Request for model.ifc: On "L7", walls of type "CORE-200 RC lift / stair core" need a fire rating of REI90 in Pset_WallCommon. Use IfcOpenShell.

First a look at what the model holds.

```python
import ifcopenshell
import ifcopenshell.util.element

model = ifcopenshell.open("model.ifc")
print(model.schema)
storey = next(s for s in model.by_type("IfcBuildingStorey") if s.Name == "L7")
walls = [e for e in ifcopenshell.util.element.get_decomposition(storey) if e.is_a("IfcWall")]
seen = {}
for e in walls:
    element_type = ifcopenshell.util.element.get_type(e)
    key = (element_type.Name if element_type != e and element_type else None, ifcopenshell.util.element.get_pset(e, "Pset_WallCommon", "FireRating"))
    seen[key] = seen.get(key, 0) + 1
for (name, value), count in sorted(seen.items(), key=str):
    print(count, "x", name, "|", value)
```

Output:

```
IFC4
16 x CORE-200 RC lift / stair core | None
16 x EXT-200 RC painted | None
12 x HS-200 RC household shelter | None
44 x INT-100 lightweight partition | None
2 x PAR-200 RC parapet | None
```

```python
import ifcopenshell
import ifcopenshell.api.pset
import ifcopenshell.util.element

model = ifcopenshell.open("model.ifc")

storey = next(s for s in model.by_type("IfcBuildingStorey") if s.Name == "L7")
walls = [e for e in ifcopenshell.util.element.get_decomposition(storey) if e.is_a("IfcWall")]

count = 0
for e in walls:
    element_type = ifcopenshell.util.element.get_type(e)
    if element_type in (None, e) or element_type.Name != "CORE-200 RC lift / stair core":
        continue
    # add_pset returns the element's existing set when there is one.
    pset = ifcopenshell.api.pset.add_pset(model, product=e, name="Pset_WallCommon")
    ifcopenshell.api.pset.edit_pset(model, pset=pset, properties={"FireRating": "REI90"})
    count += 1

print(count, "walls updated")

model.write("model-out.ifc")
```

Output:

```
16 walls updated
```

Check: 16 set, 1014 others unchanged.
